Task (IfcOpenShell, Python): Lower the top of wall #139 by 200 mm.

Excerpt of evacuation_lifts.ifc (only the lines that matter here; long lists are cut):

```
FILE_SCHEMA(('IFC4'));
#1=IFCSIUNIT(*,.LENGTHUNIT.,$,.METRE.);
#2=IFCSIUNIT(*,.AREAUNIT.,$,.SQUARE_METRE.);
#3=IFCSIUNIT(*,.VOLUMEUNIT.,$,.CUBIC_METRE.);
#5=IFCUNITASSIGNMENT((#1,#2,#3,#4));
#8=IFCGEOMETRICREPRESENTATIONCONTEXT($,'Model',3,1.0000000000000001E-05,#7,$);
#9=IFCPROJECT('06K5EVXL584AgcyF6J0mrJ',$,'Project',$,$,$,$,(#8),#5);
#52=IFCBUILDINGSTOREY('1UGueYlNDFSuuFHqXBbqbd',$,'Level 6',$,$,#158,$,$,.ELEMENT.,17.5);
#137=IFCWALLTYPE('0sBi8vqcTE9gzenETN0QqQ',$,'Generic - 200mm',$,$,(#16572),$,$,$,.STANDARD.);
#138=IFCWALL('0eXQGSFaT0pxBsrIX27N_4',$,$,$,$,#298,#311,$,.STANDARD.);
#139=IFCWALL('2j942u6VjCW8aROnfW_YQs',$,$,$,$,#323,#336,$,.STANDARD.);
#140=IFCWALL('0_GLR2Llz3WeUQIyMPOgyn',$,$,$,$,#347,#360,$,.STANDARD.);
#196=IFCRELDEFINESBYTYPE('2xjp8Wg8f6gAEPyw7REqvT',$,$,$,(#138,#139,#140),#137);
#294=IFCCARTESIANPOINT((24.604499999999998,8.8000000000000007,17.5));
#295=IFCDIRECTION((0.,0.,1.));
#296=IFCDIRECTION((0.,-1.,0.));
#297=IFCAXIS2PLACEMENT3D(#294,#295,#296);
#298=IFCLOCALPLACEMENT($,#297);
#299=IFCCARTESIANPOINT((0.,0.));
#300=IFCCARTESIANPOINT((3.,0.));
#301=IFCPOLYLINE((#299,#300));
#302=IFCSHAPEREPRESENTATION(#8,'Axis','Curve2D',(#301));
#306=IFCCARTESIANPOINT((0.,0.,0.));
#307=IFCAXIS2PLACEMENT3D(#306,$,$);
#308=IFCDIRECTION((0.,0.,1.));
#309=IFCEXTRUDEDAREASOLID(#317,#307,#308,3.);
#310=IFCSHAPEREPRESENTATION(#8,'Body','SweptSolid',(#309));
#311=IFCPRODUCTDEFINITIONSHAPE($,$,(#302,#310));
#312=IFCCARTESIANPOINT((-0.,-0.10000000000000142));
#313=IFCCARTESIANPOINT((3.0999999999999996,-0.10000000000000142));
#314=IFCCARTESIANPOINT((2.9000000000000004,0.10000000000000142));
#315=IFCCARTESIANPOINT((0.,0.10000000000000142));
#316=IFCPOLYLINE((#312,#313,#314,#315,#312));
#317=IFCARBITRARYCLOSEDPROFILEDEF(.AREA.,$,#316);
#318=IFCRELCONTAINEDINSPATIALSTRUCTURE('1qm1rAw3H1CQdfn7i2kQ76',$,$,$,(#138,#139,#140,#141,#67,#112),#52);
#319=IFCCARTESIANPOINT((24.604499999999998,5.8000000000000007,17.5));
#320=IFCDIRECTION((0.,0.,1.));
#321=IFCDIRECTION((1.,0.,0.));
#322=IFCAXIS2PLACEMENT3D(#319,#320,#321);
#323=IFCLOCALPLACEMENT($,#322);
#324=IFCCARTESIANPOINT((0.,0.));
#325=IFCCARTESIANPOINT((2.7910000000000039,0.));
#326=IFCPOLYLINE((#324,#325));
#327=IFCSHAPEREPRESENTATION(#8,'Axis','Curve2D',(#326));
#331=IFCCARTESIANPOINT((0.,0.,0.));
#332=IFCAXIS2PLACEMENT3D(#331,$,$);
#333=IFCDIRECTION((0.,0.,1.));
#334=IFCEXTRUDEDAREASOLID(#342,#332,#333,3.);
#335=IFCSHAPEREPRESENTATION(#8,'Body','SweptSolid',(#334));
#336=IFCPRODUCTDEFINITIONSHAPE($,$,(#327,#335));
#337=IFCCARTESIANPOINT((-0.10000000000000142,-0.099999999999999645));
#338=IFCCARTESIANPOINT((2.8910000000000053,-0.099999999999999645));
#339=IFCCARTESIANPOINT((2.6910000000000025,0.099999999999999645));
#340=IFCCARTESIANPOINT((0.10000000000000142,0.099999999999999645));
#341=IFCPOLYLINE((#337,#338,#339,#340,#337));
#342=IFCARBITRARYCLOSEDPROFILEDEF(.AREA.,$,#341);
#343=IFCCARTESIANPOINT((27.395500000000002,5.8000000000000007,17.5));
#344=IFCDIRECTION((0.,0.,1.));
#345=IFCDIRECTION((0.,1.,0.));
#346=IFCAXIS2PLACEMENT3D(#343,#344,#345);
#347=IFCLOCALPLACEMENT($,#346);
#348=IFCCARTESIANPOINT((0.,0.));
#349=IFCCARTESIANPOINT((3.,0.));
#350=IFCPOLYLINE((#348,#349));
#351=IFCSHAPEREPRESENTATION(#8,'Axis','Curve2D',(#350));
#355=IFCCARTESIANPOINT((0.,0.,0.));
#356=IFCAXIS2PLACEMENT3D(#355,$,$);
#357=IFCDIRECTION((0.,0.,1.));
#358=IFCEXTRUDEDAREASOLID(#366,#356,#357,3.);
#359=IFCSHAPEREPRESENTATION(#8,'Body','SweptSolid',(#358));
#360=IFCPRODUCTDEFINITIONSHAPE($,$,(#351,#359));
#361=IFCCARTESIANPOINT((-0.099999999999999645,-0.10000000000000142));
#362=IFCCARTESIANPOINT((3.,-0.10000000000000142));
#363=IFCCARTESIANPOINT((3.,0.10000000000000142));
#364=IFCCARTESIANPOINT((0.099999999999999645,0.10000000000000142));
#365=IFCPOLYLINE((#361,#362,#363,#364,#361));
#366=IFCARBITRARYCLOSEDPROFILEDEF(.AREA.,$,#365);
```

```python
import ifcopenshell
import ifcopenshell.geom
import ifcopenshell.util.shape

model = ifcopenshell.open("evacuation_lifts.ifc")
settings = ifcopenshell.geom.settings()


def volume(element):
    """Net volume in cubic metres, openings subtracted."""
    shape = ifcopenshell.geom.create_shape(settings, element)
    return ifcopenshell.util.shape.get_volume(shape.geometry)


wall = model.by_id(139)
before = volume(wall)

body = next(r for r in wall.Representation.Representations if r.RepresentationIdentifier == "Body")
solid = body.Items[0]
old_height = solid.Depth
solid.Depth -= 0.2
after = volume(wall)

print(f"height {old_height:g} -> {solid.Depth:g}, volume {before:.3f} -> {after:.3f} m3")

model.write("evacuation_lifts_edited.ifc")
```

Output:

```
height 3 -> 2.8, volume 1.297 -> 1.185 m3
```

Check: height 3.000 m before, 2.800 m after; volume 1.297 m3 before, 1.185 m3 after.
